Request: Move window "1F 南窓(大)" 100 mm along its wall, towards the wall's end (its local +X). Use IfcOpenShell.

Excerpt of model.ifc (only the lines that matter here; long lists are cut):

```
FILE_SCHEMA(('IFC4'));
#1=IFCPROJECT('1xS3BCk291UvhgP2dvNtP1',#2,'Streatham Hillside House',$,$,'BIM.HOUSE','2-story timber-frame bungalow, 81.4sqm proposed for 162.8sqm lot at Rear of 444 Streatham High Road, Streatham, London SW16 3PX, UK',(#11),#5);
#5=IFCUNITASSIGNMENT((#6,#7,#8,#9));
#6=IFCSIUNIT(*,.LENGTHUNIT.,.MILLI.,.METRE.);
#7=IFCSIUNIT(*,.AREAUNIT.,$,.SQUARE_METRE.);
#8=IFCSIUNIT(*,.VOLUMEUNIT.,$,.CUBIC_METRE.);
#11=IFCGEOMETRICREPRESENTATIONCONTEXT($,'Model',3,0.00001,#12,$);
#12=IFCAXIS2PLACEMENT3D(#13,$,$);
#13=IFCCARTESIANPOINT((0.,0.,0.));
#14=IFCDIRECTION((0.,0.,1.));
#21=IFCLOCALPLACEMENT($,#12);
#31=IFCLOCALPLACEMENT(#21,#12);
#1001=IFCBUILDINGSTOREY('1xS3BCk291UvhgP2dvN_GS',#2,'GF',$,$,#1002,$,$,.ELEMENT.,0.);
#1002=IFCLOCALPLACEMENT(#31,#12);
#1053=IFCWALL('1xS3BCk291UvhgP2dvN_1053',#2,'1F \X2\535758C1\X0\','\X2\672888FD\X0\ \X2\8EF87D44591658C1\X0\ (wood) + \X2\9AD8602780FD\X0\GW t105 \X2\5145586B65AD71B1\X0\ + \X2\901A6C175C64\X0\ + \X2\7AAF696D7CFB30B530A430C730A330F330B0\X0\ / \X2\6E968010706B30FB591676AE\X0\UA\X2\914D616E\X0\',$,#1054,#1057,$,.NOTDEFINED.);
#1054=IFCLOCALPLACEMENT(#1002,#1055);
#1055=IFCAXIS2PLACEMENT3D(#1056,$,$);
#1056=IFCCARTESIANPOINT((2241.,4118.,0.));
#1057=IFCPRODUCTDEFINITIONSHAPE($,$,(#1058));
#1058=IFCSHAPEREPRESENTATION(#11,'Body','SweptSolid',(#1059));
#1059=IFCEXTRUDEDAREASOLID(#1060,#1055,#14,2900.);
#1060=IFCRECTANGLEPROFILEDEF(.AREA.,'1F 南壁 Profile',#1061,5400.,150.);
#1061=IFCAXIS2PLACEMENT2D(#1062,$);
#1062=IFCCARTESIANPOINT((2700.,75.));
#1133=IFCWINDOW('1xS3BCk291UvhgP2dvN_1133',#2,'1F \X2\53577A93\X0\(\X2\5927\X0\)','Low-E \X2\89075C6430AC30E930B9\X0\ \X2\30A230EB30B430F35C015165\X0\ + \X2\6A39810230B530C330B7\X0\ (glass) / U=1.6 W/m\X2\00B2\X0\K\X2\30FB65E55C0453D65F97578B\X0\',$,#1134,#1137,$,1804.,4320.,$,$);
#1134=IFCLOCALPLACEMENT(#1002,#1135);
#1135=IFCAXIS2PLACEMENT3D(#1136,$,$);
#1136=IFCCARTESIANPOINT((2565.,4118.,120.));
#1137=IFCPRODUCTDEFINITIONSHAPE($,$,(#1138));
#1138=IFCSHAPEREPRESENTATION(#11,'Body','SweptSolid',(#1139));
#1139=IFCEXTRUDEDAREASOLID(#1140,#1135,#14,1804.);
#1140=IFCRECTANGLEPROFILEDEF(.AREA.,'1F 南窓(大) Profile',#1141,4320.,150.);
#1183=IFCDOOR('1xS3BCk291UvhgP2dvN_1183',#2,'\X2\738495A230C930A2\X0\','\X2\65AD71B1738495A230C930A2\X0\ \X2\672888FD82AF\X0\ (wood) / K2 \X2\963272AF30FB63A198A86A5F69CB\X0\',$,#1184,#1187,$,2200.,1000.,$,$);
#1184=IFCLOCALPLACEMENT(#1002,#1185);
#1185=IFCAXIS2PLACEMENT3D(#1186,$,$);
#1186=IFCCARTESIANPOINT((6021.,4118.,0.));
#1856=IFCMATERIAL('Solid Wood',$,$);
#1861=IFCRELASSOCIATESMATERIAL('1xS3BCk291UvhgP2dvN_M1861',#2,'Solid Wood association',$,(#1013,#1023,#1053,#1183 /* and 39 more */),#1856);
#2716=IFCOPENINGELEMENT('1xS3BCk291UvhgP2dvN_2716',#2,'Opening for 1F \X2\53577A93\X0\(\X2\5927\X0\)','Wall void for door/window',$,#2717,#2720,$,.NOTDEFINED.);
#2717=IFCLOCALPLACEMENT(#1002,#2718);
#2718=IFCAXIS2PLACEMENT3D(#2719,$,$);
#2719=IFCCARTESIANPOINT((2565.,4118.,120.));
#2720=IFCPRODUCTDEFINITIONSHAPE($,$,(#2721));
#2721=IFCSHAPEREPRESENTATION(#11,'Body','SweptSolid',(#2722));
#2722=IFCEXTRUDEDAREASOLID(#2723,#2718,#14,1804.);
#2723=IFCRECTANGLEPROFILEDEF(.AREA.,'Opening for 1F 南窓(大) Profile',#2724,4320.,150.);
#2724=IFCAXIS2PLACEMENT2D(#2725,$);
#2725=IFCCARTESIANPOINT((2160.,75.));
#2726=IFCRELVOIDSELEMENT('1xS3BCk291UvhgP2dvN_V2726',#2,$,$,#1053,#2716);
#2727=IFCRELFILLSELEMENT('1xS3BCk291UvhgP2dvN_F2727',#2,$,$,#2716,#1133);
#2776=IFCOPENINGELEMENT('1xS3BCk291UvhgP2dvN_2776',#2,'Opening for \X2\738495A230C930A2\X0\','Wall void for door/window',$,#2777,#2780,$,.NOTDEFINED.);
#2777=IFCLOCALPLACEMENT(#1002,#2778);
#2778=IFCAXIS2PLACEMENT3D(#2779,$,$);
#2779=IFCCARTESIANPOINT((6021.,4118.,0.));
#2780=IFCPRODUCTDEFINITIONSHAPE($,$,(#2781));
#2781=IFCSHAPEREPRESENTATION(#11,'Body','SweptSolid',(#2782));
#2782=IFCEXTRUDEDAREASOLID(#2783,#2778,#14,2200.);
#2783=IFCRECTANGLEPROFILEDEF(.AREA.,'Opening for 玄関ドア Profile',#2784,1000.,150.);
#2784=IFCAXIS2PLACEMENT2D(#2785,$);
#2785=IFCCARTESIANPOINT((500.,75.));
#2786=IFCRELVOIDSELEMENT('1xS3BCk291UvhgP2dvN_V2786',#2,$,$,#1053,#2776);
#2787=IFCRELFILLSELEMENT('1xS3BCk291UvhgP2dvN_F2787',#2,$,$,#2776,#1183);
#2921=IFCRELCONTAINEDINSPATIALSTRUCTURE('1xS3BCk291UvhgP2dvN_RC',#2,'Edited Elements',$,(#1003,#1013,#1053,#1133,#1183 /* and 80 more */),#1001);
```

```python
import ifcopenshell
import ifcopenshell.api.geometry
import ifcopenshell.util.placement
import ifcopenshell.util.unit

model = ifcopenshell.open("model.ifc")
unit_scale = ifcopenshell.util.unit.calculate_unit_scale(model)

window = model.by_guid("1xS3BCk291UvhgP2dvN_1133")
opening = window.FillsVoids[0].RelatingOpeningElement
wall = opening.VoidsElements[0].RelatingBuildingElement

wall_matrix = ifcopenshell.util.placement.get_local_placement(wall.ObjectPlacement)
shift = wall_matrix[:3, 0] * 0.1 / unit_scale
before = ifcopenshell.util.placement.get_local_placement(window.ObjectPlacement)[:3, 3].copy()

# The window is not placed relative to its opening, so move both.
for product in (opening, window):
    matrix = ifcopenshell.util.placement.get_local_placement(product.ObjectPlacement)
    matrix[:3, 3] += shift
    ifcopenshell.api.geometry.edit_object_placement(model, product=product, matrix=matrix, is_si=False)

after = ifcopenshell.util.placement.get_local_placement(window.ObjectPlacement)[:3, 3]
print("window moved by", (after - before).round(3) + 0.0)

model.write("model_updated.ifc")
```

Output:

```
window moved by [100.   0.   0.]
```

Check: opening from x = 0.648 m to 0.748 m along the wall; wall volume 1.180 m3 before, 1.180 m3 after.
